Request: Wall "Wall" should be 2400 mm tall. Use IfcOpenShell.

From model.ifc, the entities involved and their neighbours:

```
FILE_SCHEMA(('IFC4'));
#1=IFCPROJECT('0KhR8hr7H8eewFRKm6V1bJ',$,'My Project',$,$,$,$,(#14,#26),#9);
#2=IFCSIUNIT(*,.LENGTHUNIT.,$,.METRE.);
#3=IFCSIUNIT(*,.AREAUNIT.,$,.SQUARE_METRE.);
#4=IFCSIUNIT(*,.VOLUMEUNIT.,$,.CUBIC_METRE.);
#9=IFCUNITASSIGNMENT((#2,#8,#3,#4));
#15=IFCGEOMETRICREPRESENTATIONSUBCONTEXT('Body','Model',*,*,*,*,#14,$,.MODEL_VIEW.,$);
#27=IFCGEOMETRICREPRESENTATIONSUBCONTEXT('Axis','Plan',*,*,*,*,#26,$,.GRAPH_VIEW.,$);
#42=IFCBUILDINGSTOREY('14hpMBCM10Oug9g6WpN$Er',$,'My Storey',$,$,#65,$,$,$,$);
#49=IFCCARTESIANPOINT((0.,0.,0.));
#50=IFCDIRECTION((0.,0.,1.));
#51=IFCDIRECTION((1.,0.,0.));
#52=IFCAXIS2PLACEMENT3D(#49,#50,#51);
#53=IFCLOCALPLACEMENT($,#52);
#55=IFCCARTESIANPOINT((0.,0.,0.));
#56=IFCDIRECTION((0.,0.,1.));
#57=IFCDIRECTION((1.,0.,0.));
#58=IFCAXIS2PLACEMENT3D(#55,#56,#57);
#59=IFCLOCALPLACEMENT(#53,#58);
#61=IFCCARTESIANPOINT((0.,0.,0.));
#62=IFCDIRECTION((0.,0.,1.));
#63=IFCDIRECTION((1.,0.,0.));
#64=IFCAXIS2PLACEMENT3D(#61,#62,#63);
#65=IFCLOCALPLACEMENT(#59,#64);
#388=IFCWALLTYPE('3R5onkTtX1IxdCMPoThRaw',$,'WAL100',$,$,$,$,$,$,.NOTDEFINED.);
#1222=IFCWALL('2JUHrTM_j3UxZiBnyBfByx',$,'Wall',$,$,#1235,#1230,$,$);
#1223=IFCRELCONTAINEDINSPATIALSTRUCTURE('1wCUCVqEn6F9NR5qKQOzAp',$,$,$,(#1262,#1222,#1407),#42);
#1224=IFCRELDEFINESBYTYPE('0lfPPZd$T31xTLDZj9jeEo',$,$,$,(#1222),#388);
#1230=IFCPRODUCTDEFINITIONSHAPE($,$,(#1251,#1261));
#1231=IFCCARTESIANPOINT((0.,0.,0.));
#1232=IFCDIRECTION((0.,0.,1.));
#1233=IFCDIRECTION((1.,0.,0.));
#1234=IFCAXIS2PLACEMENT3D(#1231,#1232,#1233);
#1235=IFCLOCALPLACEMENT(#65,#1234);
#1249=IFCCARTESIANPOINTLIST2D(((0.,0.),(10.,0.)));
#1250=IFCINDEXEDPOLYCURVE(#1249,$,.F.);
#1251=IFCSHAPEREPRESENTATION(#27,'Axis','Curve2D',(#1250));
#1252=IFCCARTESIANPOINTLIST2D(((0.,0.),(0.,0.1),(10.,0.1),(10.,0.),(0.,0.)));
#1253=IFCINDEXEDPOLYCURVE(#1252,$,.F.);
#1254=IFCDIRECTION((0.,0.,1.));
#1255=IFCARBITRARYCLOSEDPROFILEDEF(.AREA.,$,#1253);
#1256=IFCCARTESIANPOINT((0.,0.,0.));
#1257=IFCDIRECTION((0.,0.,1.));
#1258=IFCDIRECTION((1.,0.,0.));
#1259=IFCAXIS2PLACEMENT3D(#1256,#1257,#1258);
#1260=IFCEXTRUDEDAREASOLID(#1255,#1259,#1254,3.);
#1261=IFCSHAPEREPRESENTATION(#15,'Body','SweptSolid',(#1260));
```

```python
import ifcopenshell
import ifcopenshell.geom
import ifcopenshell.util.representation
import ifcopenshell.util.shape
import ifcopenshell.util.unit

model = ifcopenshell.open("model.ifc")
unit_scale = ifcopenshell.util.unit.calculate_unit_scale(model)
settings = ifcopenshell.geom.settings()


def volume(element):
    """Net volume in cubic metres, openings subtracted."""
    shape = ifcopenshell.geom.create_shape(settings, element)
    return ifcopenshell.util.shape.get_volume(shape.geometry)


wall = model.by_guid("2JUHrTM_j3UxZiBnyBfByx")
before = volume(wall)

body = ifcopenshell.util.representation.get_representation(wall, "Model", "Body")
solid = body.Items[0]
old_height = solid.Depth
solid.Depth = 2.4 / unit_scale
after = volume(wall)

print(f"height {old_height:g} -> {solid.Depth:g}, volume {before:.3f} -> {after:.3f} m3")

model.write("model_v2.ifc")
```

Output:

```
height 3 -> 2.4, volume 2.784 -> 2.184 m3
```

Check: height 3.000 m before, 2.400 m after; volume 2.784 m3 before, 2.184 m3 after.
